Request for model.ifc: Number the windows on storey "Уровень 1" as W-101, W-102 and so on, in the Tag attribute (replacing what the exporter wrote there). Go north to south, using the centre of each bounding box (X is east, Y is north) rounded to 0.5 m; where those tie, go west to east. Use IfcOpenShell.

First a look at what the model holds.

```python
import ifcopenshell
import ifcopenshell.util.element
import ifcopenshell.util.placement

model = ifcopenshell.open("model.ifc")
print(model.schema)
storey = next(s for s in model.by_type("IfcBuildingStorey") if s.Name == "Уровень 1")
windows = [e for e in ifcopenshell.util.element.get_decomposition(storey) if e.is_a("IfcWindow")]
for e in sorted(windows, key=lambda e: e.id()):
    origin = ifcopenshell.util.placement.get_local_placement(e.ObjectPlacement)[:3, 3]
    print(e.id(), e.Tag, e.Name, origin.round(2) + 0.0, sep=" | ")
```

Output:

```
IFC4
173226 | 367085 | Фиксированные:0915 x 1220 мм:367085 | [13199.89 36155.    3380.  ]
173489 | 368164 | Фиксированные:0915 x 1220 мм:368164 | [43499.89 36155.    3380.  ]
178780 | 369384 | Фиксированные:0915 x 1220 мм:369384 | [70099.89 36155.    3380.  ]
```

```python
import ifcopenshell
import ifcopenshell.geom
import ifcopenshell.util.element
import ifcopenshell.util.shape

model = ifcopenshell.open("model.ifc")
settings = ifcopenshell.geom.settings()
settings.set("use-world-coords", True)


def centre(element):
    shape = ifcopenshell.geom.create_shape(settings, element)
    return ifcopenshell.util.shape.get_bbox_centroid(shape.geometry)


storey = next(s for s in model.by_type("IfcBuildingStorey") if s.Name == "Уровень 1")
windows = [e for e in ifcopenshell.util.element.get_decomposition(storey) if e.is_a("IfcWindow")]

# Insertion points can sit at a corner or the storey origin, so sort by the geometry (in metres).
centres = {e: centre(e) for e in windows}
windows.sort(key=lambda e: (-round(centres[e][1] / 0.5), centres[e][0]))

for i, e in enumerate(windows, start=1):
    number = f"W-1{i:02d}"
    e.Tag = number
    print(e.id(), number)

model.write("model_updated.ifc")
```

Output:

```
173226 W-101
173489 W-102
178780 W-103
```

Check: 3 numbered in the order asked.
